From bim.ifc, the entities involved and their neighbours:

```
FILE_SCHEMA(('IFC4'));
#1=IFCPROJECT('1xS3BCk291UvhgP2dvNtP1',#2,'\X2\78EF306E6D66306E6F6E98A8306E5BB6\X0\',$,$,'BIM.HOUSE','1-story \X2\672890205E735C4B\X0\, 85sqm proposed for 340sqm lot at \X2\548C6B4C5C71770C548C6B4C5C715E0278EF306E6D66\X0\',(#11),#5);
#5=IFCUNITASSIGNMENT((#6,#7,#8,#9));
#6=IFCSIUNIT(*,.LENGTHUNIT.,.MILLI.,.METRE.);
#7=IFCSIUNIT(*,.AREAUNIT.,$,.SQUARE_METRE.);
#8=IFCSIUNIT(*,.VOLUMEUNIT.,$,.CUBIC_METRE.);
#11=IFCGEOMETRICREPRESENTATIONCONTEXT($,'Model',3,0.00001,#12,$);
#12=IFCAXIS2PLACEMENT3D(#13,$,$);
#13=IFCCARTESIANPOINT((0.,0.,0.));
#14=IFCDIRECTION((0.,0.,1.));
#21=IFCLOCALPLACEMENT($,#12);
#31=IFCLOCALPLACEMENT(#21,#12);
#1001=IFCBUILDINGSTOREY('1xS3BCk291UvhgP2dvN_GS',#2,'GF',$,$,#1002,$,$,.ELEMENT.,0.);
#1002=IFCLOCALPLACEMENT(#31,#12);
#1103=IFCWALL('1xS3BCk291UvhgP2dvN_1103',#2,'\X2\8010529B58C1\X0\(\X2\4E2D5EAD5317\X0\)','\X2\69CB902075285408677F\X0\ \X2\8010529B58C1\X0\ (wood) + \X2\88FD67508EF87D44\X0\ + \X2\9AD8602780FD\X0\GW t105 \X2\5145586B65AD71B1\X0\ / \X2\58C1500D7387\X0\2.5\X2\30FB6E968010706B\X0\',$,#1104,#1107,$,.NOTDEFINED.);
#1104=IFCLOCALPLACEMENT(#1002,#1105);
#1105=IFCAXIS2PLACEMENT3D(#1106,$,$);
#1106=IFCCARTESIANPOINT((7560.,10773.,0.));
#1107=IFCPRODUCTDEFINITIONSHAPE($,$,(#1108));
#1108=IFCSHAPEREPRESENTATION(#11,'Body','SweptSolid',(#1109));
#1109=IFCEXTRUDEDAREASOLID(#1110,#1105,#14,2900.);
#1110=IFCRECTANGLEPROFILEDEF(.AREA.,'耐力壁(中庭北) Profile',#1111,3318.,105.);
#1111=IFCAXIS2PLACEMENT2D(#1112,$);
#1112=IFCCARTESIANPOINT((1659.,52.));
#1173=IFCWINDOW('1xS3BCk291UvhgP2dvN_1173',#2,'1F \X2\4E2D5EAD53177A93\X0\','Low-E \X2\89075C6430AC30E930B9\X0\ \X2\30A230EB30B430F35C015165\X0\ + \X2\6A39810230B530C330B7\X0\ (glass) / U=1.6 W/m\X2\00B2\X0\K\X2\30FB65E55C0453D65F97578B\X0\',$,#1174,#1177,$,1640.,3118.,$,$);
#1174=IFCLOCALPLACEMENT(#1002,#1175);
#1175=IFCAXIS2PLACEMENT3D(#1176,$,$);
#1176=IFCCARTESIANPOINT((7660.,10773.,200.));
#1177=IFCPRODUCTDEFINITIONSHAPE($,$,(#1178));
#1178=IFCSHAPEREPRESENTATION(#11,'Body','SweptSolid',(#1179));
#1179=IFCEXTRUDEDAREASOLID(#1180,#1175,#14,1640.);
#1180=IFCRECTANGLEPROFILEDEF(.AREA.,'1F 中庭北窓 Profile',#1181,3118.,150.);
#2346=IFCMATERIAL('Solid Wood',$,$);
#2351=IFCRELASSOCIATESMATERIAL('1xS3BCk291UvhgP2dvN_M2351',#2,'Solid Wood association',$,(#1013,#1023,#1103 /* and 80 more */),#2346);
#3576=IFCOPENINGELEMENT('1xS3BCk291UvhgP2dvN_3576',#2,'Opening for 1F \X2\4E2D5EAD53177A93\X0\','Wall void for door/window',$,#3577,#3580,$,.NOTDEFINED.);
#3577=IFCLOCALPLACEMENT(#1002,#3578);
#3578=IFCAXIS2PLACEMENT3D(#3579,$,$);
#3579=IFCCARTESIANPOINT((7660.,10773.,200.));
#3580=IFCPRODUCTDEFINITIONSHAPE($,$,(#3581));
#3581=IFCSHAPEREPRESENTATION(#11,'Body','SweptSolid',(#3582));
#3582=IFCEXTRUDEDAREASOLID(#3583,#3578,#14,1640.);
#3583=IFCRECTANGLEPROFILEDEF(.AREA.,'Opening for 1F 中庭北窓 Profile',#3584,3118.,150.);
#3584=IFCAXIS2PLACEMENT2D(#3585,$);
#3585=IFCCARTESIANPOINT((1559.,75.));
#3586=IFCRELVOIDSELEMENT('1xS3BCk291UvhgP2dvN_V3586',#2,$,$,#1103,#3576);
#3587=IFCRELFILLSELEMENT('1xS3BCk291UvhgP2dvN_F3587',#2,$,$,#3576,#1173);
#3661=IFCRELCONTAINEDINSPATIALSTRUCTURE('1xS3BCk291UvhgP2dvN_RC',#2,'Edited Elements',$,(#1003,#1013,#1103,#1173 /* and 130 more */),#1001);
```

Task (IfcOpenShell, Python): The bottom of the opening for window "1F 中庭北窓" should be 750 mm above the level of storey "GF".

```python
import numpy as np
import ifcopenshell
import ifcopenshell.api.geometry
import ifcopenshell.geom
import ifcopenshell.util.element
import ifcopenshell.util.placement
import ifcopenshell.util.shape
import ifcopenshell.util.unit

model = ifcopenshell.open("bim.ifc")
unit_scale = ifcopenshell.util.unit.calculate_unit_scale(model)

window = model.by_id(1173)
opening = window.FillsVoids[0].RelatingOpeningElement
storey = ifcopenshell.util.element.get_container(window, ifc_class="IfcBuildingStorey")
level = ifcopenshell.util.placement.get_local_placement(storey.ObjectPlacement)[2, 3]

# The opening's origin need not be at the sill, so measure its lowest point.
shape = ifcopenshell.geom.create_shape(ifcopenshell.geom.settings(), opening)
bottom = ifcopenshell.util.shape.get_shape_bottom_elevation(shape, shape.geometry) / unit_scale
dz = level + 0.75 / unit_scale - bottom

shift = np.array([0.0, 0.0, dz])
# The window is not placed relative to its opening, so move both.
for product in (opening, window):
    matrix = ifcopenshell.util.placement.get_local_placement(product.ObjectPlacement)
    matrix[:3, 3] += shift
    ifcopenshell.api.geometry.edit_object_placement(model, product=product, matrix=matrix, is_si=False)

print(f"moved by {dz * unit_scale:+.3f} m")

model.write("bim-out.ifc")
```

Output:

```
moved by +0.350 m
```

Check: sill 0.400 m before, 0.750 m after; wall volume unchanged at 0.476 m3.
